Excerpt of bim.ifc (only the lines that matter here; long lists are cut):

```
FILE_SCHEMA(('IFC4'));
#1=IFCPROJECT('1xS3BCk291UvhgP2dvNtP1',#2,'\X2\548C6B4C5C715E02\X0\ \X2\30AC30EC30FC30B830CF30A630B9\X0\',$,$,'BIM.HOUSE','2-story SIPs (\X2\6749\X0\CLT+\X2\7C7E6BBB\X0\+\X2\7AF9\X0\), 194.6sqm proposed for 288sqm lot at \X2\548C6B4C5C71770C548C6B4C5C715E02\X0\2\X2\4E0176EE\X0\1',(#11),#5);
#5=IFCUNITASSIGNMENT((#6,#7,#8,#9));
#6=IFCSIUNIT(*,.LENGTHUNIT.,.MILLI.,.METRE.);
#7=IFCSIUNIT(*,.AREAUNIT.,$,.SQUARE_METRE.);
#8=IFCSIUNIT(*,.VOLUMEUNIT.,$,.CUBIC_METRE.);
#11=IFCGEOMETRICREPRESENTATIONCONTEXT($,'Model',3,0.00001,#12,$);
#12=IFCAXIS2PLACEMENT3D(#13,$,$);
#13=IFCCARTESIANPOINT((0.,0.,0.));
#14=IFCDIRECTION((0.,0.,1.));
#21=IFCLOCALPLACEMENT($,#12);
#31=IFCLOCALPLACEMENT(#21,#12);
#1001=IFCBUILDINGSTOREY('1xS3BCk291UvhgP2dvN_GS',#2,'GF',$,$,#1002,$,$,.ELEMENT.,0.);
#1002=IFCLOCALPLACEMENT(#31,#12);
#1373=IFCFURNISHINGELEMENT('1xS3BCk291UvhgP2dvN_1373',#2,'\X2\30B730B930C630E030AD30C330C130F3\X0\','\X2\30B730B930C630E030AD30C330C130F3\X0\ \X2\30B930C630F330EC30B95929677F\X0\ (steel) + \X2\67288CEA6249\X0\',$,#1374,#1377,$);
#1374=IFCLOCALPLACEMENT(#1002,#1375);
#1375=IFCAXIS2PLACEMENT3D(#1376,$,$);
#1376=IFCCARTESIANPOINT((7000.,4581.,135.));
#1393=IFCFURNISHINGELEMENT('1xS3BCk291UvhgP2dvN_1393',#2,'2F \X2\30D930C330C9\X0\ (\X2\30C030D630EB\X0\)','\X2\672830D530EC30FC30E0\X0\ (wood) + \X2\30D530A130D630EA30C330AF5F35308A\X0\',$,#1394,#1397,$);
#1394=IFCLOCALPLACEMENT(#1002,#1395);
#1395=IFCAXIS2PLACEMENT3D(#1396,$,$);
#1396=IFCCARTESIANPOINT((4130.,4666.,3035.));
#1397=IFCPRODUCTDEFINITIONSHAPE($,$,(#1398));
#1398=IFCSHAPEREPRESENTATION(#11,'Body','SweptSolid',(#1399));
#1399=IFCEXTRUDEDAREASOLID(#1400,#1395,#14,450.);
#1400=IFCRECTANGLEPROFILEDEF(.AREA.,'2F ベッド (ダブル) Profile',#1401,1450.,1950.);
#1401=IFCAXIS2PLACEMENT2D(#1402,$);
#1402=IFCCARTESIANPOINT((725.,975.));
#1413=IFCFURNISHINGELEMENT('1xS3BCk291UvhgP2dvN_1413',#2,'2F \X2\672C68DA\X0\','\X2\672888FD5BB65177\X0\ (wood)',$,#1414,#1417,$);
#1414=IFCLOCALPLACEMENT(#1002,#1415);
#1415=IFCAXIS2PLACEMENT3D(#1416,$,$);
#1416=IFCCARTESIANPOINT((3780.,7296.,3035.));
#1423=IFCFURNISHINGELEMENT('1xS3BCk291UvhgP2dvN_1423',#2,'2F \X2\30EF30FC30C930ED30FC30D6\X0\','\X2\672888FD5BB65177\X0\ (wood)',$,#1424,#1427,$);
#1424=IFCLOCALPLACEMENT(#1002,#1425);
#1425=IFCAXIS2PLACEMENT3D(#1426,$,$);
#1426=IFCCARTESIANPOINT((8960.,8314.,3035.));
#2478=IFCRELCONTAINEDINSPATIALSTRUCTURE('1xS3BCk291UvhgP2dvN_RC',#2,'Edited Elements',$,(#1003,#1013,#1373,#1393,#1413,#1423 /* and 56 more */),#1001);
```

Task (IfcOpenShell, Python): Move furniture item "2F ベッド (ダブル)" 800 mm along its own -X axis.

```python
import ifcopenshell
import ifcopenshell.api.geometry
import ifcopenshell.util.placement

model = ifcopenshell.open("bim.ifc")

item = model.by_guid("1xS3BCk291UvhgP2dvN_1393")
matrix = ifcopenshell.util.placement.get_local_placement(item.ObjectPlacement)
matrix[:3, 3] -= matrix[:3, 0] * 800.0
ifcopenshell.api.geometry.edit_object_placement(model, product=item, matrix=matrix, is_si=False)

print(ifcopenshell.util.placement.get_local_placement(item.ObjectPlacement).round(3) + 0.0)

model.write("bim_updated.ifc")
```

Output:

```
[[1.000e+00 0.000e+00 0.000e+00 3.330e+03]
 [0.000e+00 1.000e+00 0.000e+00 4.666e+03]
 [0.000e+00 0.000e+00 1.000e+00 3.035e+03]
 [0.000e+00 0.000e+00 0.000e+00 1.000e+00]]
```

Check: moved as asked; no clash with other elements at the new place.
